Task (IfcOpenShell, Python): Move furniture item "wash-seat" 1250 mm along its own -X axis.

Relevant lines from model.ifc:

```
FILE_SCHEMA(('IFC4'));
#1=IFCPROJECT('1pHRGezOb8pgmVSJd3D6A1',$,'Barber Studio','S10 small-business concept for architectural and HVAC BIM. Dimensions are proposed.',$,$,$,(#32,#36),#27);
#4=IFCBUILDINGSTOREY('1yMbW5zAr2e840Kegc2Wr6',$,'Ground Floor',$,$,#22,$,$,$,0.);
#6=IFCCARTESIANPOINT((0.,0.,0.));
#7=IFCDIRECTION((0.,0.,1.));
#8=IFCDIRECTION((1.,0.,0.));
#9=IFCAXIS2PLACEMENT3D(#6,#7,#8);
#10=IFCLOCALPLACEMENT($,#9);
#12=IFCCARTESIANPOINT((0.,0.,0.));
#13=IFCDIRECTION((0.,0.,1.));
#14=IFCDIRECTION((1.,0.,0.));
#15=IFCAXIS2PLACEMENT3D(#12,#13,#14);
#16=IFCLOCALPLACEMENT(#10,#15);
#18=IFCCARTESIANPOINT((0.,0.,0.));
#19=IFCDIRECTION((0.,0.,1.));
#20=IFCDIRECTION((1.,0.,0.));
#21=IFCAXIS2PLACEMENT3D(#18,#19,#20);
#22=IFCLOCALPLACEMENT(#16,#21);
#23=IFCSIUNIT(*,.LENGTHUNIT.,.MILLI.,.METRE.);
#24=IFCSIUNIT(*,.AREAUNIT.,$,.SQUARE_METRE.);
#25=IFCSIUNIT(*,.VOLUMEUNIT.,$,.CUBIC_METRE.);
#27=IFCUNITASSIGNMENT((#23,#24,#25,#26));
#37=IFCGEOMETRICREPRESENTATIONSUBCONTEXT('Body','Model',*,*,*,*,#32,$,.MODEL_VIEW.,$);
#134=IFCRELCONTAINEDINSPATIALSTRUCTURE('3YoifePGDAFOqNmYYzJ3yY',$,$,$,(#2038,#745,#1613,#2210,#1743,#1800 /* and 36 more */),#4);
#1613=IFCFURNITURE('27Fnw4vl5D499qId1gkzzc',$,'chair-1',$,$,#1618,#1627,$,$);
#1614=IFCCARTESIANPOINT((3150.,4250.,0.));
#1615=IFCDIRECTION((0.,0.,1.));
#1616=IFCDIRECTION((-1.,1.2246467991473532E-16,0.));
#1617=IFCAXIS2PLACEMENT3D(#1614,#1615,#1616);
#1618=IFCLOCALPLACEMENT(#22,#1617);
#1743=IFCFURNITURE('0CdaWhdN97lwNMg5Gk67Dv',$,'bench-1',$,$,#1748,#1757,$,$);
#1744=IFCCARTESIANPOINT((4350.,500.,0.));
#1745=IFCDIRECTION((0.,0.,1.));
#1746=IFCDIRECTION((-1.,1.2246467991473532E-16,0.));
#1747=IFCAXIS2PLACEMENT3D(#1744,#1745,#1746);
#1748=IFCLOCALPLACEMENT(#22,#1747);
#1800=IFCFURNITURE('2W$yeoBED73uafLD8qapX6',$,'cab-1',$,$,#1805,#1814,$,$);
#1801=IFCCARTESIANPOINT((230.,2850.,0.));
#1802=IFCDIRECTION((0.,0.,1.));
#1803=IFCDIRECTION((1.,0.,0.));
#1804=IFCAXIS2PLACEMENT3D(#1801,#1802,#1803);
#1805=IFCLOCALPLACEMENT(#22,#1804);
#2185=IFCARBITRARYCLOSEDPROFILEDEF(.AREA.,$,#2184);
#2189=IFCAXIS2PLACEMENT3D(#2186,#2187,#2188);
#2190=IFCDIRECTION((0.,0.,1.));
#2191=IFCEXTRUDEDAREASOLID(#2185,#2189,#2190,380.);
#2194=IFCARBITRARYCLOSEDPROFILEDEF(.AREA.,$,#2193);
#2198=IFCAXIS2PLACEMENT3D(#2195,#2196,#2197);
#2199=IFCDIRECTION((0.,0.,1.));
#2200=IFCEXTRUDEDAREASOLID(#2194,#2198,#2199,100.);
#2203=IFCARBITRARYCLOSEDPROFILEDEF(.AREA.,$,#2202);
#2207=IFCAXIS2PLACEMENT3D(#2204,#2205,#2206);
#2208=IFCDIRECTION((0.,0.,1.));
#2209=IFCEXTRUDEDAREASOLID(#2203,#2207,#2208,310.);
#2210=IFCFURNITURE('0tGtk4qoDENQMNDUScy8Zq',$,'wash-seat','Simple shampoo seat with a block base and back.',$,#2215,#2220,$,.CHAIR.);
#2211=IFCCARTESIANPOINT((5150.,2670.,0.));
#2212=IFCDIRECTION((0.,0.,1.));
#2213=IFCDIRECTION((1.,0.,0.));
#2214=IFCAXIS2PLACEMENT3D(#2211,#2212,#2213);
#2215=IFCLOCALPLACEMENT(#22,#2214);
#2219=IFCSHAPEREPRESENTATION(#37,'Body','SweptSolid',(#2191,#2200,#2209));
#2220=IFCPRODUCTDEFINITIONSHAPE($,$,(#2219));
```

```python
import ifcopenshell
import ifcopenshell.api.geometry
import ifcopenshell.util.placement
import ifcopenshell.util.unit

model = ifcopenshell.open("model.ifc")
unit_scale = ifcopenshell.util.unit.calculate_unit_scale(model)

item = model.by_guid("0tGtk4qoDENQMNDUScy8Zq")
matrix = ifcopenshell.util.placement.get_local_placement(item.ObjectPlacement)
matrix[:3, 3] -= matrix[:3, 0] * 1.25 / unit_scale
ifcopenshell.api.geometry.edit_object_placement(model, product=item, matrix=matrix, is_si=False)

print(ifcopenshell.util.placement.get_local_placement(item.ObjectPlacement).round(3) + 0.0)

model.write("model_edited.ifc")
```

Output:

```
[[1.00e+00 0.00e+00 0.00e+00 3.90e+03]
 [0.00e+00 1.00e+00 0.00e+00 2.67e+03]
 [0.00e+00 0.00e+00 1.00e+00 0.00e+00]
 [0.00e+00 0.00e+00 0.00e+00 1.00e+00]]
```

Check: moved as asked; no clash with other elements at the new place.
